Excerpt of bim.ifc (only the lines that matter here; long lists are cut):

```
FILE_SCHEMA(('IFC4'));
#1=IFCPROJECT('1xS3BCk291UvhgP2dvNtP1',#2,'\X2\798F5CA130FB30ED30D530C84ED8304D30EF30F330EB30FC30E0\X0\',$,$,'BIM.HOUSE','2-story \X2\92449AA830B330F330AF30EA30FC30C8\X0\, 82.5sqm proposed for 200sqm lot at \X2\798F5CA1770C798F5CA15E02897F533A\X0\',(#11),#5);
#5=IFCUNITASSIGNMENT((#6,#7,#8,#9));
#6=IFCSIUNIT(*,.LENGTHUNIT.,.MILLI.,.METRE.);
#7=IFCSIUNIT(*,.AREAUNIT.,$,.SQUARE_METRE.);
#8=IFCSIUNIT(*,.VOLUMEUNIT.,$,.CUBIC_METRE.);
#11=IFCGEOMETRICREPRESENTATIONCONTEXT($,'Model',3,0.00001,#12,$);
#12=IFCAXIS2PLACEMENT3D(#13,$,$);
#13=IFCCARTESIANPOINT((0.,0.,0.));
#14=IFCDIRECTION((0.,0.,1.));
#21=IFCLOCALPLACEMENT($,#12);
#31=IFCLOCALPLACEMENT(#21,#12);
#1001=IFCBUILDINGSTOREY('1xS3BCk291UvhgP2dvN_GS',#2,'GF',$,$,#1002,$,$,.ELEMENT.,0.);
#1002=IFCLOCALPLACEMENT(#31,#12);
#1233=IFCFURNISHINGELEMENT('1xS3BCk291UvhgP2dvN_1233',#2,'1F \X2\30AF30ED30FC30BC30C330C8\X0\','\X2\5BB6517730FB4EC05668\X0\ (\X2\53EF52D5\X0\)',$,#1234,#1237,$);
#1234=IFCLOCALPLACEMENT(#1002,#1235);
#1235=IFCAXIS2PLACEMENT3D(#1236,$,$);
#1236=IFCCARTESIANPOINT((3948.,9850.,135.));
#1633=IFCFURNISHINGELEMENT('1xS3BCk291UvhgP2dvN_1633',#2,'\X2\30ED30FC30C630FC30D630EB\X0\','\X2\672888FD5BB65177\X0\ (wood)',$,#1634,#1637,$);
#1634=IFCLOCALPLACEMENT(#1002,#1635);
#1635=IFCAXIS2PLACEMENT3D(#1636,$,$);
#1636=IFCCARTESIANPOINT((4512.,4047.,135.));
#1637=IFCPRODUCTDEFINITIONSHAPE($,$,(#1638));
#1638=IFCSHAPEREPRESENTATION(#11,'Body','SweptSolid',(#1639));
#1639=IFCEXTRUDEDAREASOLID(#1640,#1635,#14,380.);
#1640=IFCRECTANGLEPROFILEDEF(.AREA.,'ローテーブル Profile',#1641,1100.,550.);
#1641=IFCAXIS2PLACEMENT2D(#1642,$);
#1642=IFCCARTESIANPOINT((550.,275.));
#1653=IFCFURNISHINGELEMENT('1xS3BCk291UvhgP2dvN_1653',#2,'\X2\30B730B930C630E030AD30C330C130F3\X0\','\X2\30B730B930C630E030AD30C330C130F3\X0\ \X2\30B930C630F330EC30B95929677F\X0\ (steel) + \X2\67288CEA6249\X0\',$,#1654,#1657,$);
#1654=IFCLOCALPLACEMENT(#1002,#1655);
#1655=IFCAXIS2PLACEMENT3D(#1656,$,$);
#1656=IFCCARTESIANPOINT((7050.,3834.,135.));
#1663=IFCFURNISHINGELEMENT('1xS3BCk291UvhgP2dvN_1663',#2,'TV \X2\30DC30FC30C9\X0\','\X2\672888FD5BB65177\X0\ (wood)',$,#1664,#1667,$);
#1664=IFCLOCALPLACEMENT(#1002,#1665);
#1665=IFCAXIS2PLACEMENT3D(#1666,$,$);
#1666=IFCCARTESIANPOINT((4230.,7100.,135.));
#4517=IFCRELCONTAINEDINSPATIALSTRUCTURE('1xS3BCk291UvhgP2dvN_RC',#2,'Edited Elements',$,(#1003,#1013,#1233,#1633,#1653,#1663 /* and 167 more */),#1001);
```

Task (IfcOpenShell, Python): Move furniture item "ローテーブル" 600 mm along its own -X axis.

```python
import ifcopenshell
import ifcopenshell.api.geometry
import ifcopenshell.util.placement
import ifcopenshell.util.unit

model = ifcopenshell.open("bim.ifc")
unit_scale = ifcopenshell.util.unit.calculate_unit_scale(model)

item = model.by_guid("1xS3BCk291UvhgP2dvN_1633")
matrix = ifcopenshell.util.placement.get_local_placement(item.ObjectPlacement)
matrix[:3, 3] -= matrix[:3, 0] * 0.6 / unit_scale
ifcopenshell.api.geometry.edit_object_placement(model, product=item, matrix=matrix, is_si=False)

print(ifcopenshell.util.placement.get_local_placement(item.ObjectPlacement).round(3) + 0.0)

model.write("bim_v2.ifc")
```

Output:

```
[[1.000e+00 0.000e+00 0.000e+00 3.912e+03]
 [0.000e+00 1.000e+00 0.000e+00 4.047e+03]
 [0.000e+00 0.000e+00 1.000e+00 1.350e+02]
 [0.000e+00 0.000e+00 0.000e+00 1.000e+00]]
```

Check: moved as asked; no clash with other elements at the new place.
